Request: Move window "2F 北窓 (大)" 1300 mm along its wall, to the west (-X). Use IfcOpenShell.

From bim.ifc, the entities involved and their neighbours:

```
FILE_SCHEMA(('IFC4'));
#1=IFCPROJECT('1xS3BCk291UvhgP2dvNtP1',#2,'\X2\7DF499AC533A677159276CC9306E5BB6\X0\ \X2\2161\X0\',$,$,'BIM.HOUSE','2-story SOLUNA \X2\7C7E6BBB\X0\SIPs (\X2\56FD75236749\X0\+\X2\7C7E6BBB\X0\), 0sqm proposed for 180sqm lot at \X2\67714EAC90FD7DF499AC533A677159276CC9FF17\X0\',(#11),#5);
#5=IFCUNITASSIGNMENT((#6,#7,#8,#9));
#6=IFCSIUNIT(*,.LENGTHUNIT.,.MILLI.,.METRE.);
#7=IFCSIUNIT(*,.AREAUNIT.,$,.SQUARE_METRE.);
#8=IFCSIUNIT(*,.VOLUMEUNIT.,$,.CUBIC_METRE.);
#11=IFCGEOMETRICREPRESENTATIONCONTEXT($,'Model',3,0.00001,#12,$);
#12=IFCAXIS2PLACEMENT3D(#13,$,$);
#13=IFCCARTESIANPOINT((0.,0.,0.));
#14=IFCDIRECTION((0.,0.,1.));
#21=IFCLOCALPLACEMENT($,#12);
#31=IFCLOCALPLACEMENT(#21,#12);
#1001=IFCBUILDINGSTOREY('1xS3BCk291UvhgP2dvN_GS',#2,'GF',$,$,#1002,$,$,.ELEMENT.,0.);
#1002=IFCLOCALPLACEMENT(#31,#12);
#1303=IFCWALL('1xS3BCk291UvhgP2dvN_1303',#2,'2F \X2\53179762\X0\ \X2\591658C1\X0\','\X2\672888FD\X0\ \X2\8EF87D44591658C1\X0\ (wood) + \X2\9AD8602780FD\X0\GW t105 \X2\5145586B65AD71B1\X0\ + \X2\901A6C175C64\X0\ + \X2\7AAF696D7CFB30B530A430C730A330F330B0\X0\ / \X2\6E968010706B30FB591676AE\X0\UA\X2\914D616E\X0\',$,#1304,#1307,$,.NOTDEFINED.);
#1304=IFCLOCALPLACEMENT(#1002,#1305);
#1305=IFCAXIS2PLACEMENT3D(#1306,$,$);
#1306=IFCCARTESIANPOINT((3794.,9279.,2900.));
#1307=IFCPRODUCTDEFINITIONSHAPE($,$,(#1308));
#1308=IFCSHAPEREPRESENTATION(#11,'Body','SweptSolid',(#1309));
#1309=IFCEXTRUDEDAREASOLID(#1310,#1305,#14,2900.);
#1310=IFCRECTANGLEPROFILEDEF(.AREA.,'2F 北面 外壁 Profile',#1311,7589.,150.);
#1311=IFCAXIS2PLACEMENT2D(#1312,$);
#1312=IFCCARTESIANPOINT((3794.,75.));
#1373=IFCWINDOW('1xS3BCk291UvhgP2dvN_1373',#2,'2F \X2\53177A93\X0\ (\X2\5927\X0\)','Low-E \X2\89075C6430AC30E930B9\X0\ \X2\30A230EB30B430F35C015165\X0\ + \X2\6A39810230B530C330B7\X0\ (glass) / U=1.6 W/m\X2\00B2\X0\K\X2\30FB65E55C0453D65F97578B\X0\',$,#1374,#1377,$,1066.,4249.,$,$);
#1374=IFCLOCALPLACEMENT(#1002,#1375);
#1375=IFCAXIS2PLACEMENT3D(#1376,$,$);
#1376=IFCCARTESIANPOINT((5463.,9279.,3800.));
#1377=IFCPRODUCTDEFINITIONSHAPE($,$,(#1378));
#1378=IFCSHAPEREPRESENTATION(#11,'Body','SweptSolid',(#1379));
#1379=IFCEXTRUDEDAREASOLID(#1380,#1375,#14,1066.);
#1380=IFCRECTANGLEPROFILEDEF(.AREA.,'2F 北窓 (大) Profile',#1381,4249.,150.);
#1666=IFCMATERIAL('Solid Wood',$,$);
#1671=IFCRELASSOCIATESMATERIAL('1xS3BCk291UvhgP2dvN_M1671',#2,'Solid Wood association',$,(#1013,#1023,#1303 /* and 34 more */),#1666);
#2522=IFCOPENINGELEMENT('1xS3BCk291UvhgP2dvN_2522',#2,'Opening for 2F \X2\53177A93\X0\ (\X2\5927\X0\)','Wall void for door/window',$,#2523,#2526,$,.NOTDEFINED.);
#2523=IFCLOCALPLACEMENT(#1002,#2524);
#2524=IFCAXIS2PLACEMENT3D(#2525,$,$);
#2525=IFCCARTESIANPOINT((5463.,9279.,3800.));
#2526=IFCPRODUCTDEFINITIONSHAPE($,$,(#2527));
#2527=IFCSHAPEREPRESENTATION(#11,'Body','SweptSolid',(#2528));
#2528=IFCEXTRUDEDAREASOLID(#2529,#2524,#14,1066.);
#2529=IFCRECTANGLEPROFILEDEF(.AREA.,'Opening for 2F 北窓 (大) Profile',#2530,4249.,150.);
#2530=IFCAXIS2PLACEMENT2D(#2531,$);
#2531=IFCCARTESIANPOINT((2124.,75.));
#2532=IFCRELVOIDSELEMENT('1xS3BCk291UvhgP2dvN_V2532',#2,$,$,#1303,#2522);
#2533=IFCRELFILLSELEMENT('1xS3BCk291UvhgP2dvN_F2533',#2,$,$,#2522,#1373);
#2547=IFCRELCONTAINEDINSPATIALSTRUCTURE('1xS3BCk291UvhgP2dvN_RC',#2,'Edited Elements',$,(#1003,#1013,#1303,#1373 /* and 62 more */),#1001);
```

```python
import ifcopenshell
import ifcopenshell.api.geometry
import ifcopenshell.util.placement
import ifcopenshell.util.unit

model = ifcopenshell.open("bim.ifc")
unit_scale = ifcopenshell.util.unit.calculate_unit_scale(model)

window = model.by_guid("1xS3BCk291UvhgP2dvN_1373")
opening = window.FillsVoids[0].RelatingOpeningElement
wall = opening.VoidsElements[0].RelatingBuildingElement

wall_matrix = ifcopenshell.util.placement.get_local_placement(wall.ObjectPlacement)
shift = wall_matrix[:3, 0] * -1.3 / unit_scale
before = ifcopenshell.util.placement.get_local_placement(window.ObjectPlacement)[:3, 3].copy()

# The window is not placed relative to its opening, so move both.
for product in (opening, window):
    matrix = ifcopenshell.util.placement.get_local_placement(product.ObjectPlacement)
    matrix[:3, 3] += shift
    ifcopenshell.api.geometry.edit_object_placement(model, product=product, matrix=matrix, is_si=False)

after = ifcopenshell.util.placement.get_local_placement(window.ObjectPlacement)[:3, 3]
print("window moved by", (after - before).round(3) + 0.0)

model.write("bim_v2.ifc")
```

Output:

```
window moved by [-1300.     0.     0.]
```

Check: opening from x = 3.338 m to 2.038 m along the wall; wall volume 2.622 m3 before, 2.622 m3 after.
